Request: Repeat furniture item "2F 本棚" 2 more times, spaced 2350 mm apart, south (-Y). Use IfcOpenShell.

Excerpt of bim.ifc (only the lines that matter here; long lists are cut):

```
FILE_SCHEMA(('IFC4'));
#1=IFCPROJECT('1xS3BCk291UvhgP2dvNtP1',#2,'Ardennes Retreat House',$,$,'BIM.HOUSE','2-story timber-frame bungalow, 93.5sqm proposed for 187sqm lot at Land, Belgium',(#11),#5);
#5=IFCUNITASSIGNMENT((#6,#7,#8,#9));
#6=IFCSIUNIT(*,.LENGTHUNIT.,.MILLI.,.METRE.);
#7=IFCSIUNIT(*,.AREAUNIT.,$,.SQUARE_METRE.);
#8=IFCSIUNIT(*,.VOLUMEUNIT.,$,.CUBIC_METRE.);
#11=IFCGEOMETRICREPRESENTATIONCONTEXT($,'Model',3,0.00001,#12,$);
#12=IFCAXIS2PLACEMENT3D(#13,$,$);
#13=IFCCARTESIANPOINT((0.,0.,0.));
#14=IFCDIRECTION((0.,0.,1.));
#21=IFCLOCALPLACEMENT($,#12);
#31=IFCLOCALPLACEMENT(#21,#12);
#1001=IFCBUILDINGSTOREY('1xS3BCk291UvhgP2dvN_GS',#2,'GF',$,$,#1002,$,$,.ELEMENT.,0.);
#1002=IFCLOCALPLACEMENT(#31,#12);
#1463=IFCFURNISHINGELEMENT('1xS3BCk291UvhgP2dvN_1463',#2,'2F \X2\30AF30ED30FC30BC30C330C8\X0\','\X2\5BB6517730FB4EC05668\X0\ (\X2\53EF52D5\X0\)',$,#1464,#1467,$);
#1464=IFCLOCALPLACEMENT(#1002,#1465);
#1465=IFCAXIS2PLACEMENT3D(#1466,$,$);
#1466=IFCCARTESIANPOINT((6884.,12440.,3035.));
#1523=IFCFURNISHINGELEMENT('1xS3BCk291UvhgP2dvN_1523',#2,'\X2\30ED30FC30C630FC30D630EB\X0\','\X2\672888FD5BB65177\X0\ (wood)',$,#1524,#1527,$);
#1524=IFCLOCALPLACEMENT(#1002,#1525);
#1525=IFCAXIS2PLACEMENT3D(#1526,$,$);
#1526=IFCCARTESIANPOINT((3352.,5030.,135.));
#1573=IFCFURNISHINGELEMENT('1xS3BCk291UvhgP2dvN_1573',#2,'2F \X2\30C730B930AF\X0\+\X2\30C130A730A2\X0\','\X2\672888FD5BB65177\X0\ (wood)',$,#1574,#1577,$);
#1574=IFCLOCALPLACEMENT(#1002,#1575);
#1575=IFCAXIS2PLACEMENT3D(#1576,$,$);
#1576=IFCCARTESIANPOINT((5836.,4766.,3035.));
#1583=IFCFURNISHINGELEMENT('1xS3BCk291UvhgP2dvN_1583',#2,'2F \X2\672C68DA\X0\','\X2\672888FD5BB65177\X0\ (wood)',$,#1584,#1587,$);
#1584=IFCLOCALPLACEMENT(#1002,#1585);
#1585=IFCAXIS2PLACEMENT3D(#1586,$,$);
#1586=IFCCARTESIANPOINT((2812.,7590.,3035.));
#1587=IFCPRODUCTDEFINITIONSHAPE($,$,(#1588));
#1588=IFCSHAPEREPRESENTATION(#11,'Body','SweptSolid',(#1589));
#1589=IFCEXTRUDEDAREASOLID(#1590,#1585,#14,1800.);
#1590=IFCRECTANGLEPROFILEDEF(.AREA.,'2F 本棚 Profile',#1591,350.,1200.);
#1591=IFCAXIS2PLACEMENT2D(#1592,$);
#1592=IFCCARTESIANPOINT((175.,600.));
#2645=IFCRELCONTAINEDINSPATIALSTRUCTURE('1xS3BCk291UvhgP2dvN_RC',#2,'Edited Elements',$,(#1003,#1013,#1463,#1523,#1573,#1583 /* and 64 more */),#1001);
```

```python
import numpy as np
import ifcopenshell
import ifcopenshell.api.geometry
import ifcopenshell.api.root
import ifcopenshell.util.element
import ifcopenshell.util.placement

model = ifcopenshell.open("bim.ifc")


def reuse_history(source, copy):
    """copy_class also copies each property set's owner history, people and application; keep the originals."""
    for rel in copy.IsDefinedBy:
        if rel.is_a("IfcRelDefinesByProperties") and (history := rel.RelatingPropertyDefinition.OwnerHistory):
            rel.RelatingPropertyDefinition.OwnerHistory = source.OwnerHistory
            ifcopenshell.util.element.remove_deep2(model, history)


source = model.by_guid("1xS3BCk291UvhgP2dvN_1583")
base = ifcopenshell.util.placement.get_local_placement(source.ObjectPlacement)
step = np.array([0.0, -1.0, 0.0]) * 2350.0

for i in range(1, 3):
    copy = ifcopenshell.api.root.copy_class(model, product=source)
    copy.Representation = ifcopenshell.util.element.copy_deep(
        model, source.Representation, exclude=["IfcGeometricRepresentationContext", "IfcRepresentationMap"]
    )
    reuse_history(source, copy)
    matrix = base.copy()
    matrix[:3, 3] += i * step
    print("added at", matrix[:3, 3].round(3) + 0.0)
    ifcopenshell.api.geometry.edit_object_placement(model, product=copy, matrix=matrix, is_si=False)

model.write("bim-out.ifc")
```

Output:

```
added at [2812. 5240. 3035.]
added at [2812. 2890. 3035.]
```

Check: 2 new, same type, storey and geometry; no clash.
